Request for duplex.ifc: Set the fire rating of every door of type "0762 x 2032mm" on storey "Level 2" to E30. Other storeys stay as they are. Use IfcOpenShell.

First a look at what the model holds.

```python
import ifcopenshell
import ifcopenshell.util.element

model = ifcopenshell.open("duplex.ifc")
print(model.schema)
storey = next(s for s in model.by_type("IfcBuildingStorey") if s.Name == "Level 2")
doors = [e for e in ifcopenshell.util.element.get_decomposition(storey) if e.is_a("IfcDoor")]
seen = {}
for e in doors:
    element_type = ifcopenshell.util.element.get_type(e)
    key = (element_type.Name if element_type != e and element_type else None, ifcopenshell.util.element.get_pset(e, "Pset_DoorCommon", "FireRating"))
    seen[key] = seen.get(key, 0) + 1
for (name, value), count in sorted(seen.items(), key=str):
    print(count, "x", name, "|", value)
```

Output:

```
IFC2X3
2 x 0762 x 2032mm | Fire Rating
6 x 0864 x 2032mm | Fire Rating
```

```python
import ifcopenshell
import ifcopenshell.api.pset
import ifcopenshell.util.element

model = ifcopenshell.open("duplex.ifc")

storey = next(s for s in model.by_type("IfcBuildingStorey") if s.Name == "Level 2")
doors = [e for e in ifcopenshell.util.element.get_decomposition(storey) if e.is_a("IfcDoor")]

count = 0
for e in doors:
    element_type = ifcopenshell.util.element.get_type(e)
    if element_type in (None, e) or element_type.Name != "0762 x 2032mm":
        continue
    # add_pset returns the element's existing set when there is one.
    pset = ifcopenshell.api.pset.add_pset(model, product=e, name="Pset_DoorCommon")
    ifcopenshell.api.pset.edit_pset(model, pset=pset, properties={"FireRating": "E30"})
    count += 1

print(count, "doors updated")

model.write("duplex_edited.ifc")
```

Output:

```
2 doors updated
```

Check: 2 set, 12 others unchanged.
